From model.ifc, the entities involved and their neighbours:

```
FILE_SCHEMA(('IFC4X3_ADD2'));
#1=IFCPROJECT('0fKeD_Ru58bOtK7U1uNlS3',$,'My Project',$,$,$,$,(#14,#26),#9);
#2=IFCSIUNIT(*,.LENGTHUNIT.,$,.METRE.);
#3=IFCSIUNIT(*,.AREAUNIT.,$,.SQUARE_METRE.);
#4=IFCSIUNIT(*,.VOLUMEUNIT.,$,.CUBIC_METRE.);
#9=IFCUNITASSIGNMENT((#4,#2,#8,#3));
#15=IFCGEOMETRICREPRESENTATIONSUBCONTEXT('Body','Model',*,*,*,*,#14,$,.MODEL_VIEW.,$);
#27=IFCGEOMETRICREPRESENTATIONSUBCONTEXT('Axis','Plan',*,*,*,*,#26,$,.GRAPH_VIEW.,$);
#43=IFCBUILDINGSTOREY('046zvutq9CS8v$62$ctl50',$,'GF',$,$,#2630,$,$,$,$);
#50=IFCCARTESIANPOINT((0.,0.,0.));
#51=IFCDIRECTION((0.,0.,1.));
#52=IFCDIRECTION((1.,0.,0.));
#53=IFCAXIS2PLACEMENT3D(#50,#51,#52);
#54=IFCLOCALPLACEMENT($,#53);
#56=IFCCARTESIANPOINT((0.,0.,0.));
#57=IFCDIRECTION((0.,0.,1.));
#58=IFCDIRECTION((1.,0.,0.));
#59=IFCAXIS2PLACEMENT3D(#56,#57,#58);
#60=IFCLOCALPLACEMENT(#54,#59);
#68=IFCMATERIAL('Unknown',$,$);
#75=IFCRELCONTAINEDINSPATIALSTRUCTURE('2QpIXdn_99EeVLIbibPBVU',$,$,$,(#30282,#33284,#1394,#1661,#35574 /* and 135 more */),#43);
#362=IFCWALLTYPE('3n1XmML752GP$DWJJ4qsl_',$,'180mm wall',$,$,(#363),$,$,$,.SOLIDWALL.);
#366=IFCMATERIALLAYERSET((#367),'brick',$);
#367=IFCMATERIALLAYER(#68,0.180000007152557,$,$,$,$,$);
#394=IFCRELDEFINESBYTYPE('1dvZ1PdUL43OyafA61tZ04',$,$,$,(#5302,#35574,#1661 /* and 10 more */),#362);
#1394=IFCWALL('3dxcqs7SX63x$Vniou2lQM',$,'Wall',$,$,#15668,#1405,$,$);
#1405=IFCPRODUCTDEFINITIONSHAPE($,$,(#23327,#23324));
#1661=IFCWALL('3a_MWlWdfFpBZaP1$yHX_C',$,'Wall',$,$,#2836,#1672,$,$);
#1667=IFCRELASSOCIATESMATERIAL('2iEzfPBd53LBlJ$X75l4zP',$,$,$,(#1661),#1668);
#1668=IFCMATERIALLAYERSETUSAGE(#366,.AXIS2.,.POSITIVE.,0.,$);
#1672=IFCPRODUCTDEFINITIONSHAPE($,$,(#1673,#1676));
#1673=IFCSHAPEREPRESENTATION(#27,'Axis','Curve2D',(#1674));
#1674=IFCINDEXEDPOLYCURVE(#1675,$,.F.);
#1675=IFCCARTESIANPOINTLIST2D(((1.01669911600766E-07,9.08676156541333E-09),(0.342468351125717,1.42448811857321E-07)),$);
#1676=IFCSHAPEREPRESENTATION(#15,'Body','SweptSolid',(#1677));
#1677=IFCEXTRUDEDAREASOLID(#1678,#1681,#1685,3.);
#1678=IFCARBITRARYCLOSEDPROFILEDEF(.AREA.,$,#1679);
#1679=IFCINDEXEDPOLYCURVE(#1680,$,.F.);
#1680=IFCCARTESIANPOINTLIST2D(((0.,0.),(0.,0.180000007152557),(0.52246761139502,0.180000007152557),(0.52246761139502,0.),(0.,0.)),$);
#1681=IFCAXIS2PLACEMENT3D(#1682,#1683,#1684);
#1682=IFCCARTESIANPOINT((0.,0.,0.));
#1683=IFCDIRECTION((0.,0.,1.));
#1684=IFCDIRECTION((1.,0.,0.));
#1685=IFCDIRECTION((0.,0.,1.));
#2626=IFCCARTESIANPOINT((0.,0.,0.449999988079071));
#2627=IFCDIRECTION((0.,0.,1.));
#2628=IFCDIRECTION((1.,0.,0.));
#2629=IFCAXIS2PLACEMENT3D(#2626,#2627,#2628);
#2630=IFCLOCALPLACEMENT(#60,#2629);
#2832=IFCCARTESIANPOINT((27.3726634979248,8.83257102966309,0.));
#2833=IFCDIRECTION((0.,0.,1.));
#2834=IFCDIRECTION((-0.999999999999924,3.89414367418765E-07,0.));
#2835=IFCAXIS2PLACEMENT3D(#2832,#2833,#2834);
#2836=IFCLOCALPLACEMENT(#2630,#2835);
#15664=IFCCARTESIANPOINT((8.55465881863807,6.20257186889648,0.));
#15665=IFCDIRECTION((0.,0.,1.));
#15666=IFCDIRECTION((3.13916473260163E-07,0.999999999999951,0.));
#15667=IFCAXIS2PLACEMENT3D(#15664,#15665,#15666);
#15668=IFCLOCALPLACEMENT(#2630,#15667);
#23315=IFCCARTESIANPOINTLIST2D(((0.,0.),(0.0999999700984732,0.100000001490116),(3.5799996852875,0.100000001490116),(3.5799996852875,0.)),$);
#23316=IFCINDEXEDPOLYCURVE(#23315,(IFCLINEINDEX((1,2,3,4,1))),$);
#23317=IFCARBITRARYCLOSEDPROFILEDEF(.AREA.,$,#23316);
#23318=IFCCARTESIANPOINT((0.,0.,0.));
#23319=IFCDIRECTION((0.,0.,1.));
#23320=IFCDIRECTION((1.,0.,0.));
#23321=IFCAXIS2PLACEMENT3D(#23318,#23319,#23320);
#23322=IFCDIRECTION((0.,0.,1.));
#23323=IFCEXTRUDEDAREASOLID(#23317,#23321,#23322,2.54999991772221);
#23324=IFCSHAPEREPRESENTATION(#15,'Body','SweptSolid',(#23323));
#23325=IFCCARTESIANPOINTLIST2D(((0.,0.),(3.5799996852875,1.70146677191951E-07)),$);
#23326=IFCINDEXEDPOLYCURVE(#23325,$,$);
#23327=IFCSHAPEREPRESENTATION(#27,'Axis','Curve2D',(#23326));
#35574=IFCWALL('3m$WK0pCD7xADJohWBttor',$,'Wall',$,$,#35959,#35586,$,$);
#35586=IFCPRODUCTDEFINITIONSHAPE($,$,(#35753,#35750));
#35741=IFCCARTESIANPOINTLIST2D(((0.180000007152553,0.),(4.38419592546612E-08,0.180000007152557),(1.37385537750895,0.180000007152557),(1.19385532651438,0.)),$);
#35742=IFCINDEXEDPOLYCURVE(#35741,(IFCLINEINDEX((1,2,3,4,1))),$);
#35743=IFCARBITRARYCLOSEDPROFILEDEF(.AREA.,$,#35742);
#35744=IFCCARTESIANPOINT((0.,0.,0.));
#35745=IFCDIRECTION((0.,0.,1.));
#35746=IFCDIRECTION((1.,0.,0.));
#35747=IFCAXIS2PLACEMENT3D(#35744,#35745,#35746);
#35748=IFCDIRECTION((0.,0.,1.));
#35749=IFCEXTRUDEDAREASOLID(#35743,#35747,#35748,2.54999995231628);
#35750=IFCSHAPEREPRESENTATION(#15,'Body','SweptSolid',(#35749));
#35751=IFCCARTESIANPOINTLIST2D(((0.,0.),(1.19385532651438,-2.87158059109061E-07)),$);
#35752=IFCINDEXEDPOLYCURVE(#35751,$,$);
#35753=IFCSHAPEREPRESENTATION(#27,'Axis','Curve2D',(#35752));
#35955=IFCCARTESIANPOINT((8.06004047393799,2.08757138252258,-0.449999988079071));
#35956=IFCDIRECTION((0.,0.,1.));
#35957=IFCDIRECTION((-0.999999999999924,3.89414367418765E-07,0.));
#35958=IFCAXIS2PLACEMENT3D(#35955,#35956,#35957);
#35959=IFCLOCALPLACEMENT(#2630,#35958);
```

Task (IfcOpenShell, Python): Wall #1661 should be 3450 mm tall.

```python
import ifcopenshell
import ifcopenshell.geom
import ifcopenshell.util.representation
import ifcopenshell.util.shape

model = ifcopenshell.open("model.ifc")
settings = ifcopenshell.geom.settings()


def volume(element):
    """Net volume in cubic metres, openings subtracted."""
    shape = ifcopenshell.geom.create_shape(settings, element)
    return ifcopenshell.util.shape.get_volume(shape.geometry)


wall = model.by_guid("3a_MWlWdfFpBZaP1$yHX_C")
before = volume(wall)

body = ifcopenshell.util.representation.get_representation(wall, "Model", "Body")
solid = body.Items[0]
old_height = solid.Depth
solid.Depth = 3.45
after = volume(wall)

print(f"height {old_height:g} -> {solid.Depth:g}, volume {before:.3f} -> {after:.3f} m3")

model.write("model_v2.ifc")
```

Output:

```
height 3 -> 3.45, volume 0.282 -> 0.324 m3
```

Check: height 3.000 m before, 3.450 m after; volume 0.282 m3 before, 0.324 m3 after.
